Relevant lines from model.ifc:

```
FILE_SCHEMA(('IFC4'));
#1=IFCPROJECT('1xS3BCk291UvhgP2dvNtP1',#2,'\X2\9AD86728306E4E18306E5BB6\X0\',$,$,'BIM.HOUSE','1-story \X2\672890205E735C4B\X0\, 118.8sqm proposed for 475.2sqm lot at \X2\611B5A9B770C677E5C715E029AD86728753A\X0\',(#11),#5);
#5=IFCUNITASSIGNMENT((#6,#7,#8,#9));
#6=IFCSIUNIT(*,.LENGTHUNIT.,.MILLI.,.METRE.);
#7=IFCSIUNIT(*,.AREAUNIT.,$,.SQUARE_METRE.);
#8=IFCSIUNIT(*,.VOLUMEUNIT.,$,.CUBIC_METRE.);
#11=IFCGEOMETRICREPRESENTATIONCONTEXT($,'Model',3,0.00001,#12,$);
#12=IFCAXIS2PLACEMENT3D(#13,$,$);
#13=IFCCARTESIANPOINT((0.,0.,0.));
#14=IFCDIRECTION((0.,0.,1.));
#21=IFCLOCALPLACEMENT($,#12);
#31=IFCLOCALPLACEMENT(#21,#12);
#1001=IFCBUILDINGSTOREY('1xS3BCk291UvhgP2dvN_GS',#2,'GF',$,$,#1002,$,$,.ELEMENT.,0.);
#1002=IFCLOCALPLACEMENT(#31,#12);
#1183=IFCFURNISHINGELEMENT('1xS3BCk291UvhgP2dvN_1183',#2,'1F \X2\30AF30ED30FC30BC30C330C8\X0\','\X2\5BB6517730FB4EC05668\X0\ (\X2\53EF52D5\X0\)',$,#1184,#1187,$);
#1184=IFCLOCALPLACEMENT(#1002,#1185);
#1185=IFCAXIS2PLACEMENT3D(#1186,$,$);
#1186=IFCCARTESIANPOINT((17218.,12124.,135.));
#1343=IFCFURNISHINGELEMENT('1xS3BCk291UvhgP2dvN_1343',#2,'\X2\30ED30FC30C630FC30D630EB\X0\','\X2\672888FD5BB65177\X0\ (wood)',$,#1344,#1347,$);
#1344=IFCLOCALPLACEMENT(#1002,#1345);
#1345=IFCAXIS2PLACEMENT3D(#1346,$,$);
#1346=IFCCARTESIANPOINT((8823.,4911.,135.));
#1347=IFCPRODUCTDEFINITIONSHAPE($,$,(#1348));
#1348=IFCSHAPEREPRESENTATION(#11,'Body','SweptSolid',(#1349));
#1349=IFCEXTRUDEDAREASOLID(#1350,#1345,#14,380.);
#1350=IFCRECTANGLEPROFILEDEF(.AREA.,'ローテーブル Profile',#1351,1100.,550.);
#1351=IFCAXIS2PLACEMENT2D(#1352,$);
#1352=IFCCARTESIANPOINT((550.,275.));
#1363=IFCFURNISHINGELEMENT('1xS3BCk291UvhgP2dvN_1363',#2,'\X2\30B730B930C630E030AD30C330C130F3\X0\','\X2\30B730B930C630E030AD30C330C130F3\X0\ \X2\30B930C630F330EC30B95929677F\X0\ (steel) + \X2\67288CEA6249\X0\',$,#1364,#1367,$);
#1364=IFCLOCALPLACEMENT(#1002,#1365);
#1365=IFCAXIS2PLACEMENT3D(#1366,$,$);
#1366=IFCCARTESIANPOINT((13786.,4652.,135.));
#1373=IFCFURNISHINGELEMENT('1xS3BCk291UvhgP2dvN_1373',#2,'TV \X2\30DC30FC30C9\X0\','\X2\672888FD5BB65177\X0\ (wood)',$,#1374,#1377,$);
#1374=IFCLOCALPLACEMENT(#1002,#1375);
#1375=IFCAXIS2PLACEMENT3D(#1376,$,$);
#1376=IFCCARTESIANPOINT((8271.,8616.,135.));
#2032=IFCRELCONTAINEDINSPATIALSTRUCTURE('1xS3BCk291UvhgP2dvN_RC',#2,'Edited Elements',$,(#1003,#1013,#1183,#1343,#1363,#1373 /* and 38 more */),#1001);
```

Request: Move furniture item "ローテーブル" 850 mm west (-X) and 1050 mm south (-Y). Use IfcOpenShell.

```python
import ifcopenshell
import ifcopenshell.api.geometry
import ifcopenshell.util.placement
import ifcopenshell.util.unit

model = ifcopenshell.open("model.ifc")
unit_scale = ifcopenshell.util.unit.calculate_unit_scale(model)

item = model.by_guid("1xS3BCk291UvhgP2dvN_1343")
matrix = ifcopenshell.util.placement.get_local_placement(item.ObjectPlacement)
matrix[0, 3] -= 0.85 / unit_scale
matrix[1, 3] -= 1.05 / unit_scale
ifcopenshell.api.geometry.edit_object_placement(model, product=item, matrix=matrix, is_si=False)

print(ifcopenshell.util.placement.get_local_placement(item.ObjectPlacement).round(3) + 0.0)

model.write("model_rev.ifc")
```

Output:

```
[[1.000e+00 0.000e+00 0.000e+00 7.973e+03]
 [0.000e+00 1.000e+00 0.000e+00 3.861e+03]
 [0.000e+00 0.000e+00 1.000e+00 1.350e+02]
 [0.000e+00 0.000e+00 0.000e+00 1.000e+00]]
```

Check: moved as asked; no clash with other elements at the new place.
